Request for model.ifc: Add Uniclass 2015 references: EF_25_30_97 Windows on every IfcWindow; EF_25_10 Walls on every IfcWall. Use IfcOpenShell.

First a look at what the model holds.

```python
import ifcopenshell

model = ifcopenshell.open("model.ifc")
print(model.schema)
print("classifications:", [c.Name for c in model.by_type("IfcClassification")])
for ifc_class in ("IfcDoor", "IfcRoof", "IfcStair", "IfcWall", "IfcWindow"):
    print(ifc_class, len(model.by_type(ifc_class)))
```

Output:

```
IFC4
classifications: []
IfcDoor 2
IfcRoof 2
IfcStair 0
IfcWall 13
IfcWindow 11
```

```python
import ifcopenshell
import ifcopenshell.api.classification

model = ifcopenshell.open("model.ifc")

system = ifcopenshell.api.classification.add_classification(model, classification="Uniclass 2015")

codes = {
    "IfcWindow": ("EF_25_30_97", "Windows"),
    "IfcWall": ("EF_25_10", "Walls"),
}
for ifc_class, (code, name) in codes.items():
    products = model.by_type(ifc_class)
    ifcopenshell.api.classification.add_reference(
        model, products=products, classification=system, identification=code, name=name
    )
    print(code, len(products))

model.write("model_v2.ifc")
```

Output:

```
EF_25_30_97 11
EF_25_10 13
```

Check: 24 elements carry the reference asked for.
